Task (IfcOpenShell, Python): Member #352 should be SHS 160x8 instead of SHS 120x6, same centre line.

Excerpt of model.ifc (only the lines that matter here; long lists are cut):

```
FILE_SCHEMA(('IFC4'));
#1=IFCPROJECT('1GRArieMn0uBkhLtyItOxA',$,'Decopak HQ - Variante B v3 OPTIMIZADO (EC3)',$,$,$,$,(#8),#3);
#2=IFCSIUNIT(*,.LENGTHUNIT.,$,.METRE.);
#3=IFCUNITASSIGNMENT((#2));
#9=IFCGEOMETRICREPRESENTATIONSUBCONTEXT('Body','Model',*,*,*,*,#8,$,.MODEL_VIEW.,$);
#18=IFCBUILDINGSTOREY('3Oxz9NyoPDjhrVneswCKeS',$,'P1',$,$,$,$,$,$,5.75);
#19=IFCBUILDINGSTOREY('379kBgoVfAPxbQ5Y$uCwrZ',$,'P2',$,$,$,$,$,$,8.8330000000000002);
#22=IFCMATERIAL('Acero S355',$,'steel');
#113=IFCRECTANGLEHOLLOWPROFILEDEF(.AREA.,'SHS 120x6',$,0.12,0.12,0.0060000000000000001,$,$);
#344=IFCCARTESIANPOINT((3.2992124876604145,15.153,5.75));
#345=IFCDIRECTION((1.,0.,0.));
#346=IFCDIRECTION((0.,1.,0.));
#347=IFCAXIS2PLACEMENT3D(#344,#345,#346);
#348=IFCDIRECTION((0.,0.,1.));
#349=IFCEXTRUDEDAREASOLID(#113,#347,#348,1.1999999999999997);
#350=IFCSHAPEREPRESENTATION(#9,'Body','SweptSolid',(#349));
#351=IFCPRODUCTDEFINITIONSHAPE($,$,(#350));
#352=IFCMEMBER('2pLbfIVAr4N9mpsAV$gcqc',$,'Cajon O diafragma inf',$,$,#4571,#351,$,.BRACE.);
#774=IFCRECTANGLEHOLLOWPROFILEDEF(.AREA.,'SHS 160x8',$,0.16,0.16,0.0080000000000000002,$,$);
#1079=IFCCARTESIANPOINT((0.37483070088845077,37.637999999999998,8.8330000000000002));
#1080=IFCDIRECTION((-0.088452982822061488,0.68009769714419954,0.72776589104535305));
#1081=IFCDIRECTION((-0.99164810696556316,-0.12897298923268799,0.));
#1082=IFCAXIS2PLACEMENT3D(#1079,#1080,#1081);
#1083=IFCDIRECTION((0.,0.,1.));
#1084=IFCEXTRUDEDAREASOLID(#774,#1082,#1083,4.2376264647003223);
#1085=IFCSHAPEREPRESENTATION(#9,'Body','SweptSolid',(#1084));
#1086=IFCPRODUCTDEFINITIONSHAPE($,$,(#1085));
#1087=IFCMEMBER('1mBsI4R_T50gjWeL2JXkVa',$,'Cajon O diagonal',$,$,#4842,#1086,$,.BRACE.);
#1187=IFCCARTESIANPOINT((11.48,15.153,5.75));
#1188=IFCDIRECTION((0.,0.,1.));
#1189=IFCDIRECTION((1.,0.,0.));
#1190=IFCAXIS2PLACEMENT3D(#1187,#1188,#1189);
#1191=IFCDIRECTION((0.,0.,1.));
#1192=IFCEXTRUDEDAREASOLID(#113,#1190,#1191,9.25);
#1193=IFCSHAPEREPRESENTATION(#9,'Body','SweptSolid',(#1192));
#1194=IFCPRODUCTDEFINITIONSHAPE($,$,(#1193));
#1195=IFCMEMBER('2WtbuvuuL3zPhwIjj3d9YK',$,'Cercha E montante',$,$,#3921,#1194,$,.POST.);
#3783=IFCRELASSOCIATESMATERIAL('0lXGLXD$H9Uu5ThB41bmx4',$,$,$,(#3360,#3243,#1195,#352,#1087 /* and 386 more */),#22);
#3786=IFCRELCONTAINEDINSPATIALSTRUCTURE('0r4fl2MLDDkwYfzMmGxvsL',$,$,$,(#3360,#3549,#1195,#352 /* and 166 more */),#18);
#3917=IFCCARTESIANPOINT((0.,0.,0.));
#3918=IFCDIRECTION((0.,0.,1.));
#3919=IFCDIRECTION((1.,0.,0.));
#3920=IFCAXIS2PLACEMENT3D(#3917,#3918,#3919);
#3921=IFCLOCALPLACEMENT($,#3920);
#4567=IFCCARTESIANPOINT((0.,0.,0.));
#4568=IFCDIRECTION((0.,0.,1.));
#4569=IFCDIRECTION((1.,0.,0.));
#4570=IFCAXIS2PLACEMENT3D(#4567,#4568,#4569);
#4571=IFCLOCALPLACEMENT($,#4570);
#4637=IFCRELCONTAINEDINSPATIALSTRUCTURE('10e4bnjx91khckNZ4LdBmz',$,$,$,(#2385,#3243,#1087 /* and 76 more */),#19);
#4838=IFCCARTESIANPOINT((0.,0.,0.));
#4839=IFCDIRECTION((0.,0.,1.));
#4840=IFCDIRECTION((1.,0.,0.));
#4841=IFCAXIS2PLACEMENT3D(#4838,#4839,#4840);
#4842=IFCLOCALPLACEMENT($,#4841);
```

```python
import ifcopenshell
import ifcopenshell.util.element
import ifcopenshell.util.representation

model = ifcopenshell.open("model.ifc")

member = model.by_id(352)
source = next(p for p in model.by_type("IfcRectangleHollowProfileDef") if p.ProfileName == "SHS 160x8")

body = ifcopenshell.util.representation.get_representation(member, "Model", "Body")
solid = body.Items[0]
old_profile = solid.SweptArea

# Copy the section's sizes but keep this member's own profile position.
profile = ifcopenshell.util.element.copy(model, source)
profile.Position = old_profile.Position
solid.SweptArea = profile
if not model.get_total_inverses(old_profile):
    ifcopenshell.util.element.remove_deep2(model, old_profile)

print(solid.SweptArea)

model.write("model-out.ifc")
```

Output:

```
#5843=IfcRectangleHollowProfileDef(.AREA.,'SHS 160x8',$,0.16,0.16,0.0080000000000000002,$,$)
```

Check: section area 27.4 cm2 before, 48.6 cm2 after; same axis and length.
